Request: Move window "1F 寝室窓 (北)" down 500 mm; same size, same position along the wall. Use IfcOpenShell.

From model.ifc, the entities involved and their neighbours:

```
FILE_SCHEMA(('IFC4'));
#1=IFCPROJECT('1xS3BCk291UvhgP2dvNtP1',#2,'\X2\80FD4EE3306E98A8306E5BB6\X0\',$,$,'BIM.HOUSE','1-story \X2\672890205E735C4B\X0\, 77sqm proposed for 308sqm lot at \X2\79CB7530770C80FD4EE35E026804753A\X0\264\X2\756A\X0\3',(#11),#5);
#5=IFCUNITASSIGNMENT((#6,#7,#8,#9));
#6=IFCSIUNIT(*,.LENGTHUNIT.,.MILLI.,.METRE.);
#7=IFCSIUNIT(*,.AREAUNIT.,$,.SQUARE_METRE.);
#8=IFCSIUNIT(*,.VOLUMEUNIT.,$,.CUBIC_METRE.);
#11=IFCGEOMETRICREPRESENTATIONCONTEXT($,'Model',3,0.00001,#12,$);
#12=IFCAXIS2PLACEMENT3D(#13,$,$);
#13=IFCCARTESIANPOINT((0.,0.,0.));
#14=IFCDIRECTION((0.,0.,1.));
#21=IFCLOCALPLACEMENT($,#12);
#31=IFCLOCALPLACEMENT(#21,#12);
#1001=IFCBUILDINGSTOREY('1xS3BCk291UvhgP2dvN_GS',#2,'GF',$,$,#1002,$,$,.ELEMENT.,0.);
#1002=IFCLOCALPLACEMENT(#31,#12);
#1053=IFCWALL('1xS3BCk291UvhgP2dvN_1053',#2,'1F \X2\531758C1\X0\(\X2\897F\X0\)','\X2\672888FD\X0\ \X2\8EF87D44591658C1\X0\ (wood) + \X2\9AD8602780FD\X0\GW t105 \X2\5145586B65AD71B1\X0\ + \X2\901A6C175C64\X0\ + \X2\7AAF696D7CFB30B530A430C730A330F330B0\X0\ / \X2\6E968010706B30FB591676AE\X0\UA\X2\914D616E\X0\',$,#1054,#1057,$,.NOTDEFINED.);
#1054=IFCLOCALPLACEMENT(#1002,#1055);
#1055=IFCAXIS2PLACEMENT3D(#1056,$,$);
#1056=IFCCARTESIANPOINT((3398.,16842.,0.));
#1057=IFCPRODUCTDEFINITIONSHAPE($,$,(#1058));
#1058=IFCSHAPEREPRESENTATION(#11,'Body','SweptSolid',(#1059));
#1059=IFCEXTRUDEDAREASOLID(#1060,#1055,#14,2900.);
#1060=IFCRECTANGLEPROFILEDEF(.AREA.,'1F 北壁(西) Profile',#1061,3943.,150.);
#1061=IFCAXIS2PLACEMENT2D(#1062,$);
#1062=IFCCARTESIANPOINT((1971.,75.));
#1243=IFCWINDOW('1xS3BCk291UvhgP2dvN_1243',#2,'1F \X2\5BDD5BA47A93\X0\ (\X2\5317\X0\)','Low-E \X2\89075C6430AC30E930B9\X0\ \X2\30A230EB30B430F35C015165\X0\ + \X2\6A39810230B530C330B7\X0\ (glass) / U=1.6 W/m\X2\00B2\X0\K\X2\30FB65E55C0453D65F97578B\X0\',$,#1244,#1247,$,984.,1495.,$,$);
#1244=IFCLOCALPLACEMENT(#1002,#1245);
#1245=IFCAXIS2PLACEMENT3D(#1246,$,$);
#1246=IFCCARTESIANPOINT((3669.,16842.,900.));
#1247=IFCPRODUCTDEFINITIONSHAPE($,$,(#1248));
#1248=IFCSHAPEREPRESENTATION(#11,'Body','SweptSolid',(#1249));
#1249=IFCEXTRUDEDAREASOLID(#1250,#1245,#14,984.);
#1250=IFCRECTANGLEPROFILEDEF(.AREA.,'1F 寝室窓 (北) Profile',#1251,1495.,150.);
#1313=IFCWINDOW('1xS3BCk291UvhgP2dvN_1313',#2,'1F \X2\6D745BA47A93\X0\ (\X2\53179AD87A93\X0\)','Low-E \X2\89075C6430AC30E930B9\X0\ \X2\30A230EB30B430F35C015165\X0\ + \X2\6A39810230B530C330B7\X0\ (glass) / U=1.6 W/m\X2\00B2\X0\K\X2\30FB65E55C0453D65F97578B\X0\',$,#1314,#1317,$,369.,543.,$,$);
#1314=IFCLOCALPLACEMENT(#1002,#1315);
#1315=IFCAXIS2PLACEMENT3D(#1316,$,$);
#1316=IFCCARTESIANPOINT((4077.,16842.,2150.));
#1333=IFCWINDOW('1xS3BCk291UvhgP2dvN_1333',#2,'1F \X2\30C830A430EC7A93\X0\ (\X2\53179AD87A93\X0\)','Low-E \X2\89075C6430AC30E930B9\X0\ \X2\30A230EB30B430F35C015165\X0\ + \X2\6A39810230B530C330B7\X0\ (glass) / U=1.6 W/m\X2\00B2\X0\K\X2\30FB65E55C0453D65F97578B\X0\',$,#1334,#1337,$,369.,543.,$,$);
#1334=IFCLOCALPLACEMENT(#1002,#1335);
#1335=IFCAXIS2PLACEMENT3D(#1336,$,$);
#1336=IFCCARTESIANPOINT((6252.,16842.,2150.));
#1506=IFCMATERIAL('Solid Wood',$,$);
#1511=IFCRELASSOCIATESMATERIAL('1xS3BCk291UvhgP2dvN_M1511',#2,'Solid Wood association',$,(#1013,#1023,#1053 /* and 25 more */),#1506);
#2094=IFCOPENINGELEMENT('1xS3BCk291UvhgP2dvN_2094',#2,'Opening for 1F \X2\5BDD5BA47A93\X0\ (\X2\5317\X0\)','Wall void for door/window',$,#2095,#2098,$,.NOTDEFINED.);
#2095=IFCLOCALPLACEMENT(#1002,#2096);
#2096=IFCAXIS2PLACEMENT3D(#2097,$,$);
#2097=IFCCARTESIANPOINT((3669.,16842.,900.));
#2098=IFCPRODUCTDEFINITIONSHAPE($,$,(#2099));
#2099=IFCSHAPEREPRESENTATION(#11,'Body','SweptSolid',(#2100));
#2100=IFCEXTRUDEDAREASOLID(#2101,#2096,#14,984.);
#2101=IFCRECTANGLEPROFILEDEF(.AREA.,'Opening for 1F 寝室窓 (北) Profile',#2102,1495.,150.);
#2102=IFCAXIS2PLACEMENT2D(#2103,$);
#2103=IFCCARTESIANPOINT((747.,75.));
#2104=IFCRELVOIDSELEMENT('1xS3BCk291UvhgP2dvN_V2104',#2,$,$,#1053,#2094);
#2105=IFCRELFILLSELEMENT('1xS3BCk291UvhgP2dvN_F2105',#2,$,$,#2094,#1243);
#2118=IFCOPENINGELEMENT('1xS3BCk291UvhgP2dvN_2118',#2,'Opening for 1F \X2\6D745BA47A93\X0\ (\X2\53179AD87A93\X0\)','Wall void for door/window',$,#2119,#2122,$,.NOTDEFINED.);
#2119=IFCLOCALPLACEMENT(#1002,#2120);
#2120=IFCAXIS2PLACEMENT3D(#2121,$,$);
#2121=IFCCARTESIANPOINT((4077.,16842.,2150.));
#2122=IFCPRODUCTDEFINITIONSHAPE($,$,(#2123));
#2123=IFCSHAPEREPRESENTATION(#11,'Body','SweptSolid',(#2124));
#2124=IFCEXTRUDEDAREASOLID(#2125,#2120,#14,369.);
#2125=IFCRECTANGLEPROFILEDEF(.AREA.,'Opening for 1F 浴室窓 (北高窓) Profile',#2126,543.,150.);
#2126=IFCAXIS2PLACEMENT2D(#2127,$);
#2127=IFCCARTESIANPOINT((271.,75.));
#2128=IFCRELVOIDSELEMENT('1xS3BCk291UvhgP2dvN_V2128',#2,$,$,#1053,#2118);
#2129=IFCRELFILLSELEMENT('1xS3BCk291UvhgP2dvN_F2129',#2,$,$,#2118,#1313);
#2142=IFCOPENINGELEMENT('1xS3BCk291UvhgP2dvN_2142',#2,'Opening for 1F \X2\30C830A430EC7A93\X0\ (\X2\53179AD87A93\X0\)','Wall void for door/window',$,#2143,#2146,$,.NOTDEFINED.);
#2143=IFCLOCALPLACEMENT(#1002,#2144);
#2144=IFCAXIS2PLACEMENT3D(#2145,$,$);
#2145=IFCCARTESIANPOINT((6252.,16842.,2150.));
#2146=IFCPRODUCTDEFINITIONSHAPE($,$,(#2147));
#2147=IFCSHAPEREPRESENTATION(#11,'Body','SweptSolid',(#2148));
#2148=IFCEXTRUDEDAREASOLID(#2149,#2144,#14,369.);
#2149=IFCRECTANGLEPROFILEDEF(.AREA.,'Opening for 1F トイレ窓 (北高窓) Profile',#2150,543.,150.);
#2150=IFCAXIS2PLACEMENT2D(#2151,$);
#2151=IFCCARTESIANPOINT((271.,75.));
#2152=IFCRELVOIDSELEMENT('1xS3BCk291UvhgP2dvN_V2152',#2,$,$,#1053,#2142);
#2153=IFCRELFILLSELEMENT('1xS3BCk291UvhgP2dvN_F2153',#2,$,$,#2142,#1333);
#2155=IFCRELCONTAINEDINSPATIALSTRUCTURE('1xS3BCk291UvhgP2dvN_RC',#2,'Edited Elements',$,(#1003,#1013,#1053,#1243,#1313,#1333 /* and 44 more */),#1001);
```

```python
import numpy as np
import ifcopenshell
import ifcopenshell.api.geometry
import ifcopenshell.util.placement
import ifcopenshell.util.unit

model = ifcopenshell.open("model.ifc")
unit_scale = ifcopenshell.util.unit.calculate_unit_scale(model)

window = model.by_id(1243)
opening = window.FillsVoids[0].RelatingOpeningElement
dz = -0.5 / unit_scale

shift = np.array([0.0, 0.0, dz])
# The window is not placed relative to its opening, so move both.
for product in (opening, window):
    matrix = ifcopenshell.util.placement.get_local_placement(product.ObjectPlacement)
    matrix[:3, 3] += shift
    ifcopenshell.api.geometry.edit_object_placement(model, product=product, matrix=matrix, is_si=False)

print(f"moved by {dz * unit_scale:+.3f} m")

model.write("model-out.ifc")
```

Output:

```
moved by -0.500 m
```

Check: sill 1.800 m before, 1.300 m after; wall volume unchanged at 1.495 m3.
